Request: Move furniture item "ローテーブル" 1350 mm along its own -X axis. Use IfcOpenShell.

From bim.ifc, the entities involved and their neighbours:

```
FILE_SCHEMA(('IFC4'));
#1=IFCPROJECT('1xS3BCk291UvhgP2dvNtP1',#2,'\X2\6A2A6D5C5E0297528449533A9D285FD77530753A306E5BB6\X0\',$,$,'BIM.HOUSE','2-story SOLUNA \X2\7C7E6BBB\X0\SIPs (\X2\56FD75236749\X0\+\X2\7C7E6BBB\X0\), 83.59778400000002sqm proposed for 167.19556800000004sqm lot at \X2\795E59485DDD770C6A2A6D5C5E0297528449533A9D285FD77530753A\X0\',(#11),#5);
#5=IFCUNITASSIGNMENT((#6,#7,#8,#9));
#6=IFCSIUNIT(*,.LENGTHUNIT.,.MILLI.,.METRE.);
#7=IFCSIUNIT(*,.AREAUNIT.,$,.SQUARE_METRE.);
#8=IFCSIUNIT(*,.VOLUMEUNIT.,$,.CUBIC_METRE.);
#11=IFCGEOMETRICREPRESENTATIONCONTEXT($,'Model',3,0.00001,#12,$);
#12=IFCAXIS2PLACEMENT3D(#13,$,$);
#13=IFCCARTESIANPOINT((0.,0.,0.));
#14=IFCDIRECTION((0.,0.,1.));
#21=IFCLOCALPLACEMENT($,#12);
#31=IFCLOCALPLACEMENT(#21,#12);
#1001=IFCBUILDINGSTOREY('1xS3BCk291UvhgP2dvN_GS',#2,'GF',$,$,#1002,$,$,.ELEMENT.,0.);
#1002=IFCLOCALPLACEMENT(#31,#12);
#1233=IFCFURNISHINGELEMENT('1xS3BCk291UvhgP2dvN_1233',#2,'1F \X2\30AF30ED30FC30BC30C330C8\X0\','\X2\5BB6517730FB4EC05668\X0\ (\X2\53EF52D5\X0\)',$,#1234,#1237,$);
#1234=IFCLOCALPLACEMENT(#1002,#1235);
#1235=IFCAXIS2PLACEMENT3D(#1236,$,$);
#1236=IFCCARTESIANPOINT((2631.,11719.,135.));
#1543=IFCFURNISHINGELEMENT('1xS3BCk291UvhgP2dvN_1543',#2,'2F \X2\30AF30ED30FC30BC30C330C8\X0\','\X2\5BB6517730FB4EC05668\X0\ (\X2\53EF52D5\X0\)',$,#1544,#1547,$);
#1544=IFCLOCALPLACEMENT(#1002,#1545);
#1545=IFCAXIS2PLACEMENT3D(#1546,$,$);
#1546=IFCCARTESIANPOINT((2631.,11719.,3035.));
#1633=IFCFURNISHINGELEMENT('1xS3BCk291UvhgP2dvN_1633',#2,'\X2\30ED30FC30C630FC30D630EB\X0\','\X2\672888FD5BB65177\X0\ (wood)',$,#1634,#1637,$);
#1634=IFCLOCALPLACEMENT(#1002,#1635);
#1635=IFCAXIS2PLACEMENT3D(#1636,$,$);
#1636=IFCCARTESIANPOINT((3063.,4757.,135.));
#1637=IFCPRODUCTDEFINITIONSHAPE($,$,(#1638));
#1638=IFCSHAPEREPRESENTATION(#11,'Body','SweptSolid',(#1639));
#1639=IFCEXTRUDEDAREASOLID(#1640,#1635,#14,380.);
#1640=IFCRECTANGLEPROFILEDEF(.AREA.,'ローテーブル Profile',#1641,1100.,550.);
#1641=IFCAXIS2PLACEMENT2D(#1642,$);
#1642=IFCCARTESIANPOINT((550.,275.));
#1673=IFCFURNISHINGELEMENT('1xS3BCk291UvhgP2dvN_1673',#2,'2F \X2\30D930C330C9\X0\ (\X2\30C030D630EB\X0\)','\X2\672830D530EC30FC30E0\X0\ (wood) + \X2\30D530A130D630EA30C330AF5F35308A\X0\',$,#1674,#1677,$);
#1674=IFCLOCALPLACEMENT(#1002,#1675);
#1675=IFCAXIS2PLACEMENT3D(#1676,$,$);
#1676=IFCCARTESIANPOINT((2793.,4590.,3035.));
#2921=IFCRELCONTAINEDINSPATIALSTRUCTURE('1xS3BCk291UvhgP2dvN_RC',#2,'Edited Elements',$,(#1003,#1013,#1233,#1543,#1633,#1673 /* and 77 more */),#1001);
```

```python
import ifcopenshell
import ifcopenshell.api.geometry
import ifcopenshell.util.placement

model = ifcopenshell.open("bim.ifc")

item = model.by_id(1633)
matrix = ifcopenshell.util.placement.get_local_placement(item.ObjectPlacement)
matrix[:3, 3] -= matrix[:3, 0] * 1350.0
ifcopenshell.api.geometry.edit_object_placement(model, product=item, matrix=matrix, is_si=False)

print(ifcopenshell.util.placement.get_local_placement(item.ObjectPlacement).round(3) + 0.0)

model.write("bim-out.ifc")
```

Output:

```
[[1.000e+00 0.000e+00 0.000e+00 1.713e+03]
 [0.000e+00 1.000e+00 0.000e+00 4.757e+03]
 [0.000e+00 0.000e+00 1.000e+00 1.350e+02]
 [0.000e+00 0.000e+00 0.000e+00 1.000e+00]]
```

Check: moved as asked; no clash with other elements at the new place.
